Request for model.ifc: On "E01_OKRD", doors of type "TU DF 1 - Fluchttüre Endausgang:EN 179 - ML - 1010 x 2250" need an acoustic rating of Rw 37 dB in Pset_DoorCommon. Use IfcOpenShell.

First a look at what the model holds.

```python
import ifcopenshell
import ifcopenshell.util.element

model = ifcopenshell.open("model.ifc")
print(model.schema)
storey = next(s for s in model.by_type("IfcBuildingStorey") if s.Name == "E01_OKRD")
doors = [e for e in ifcopenshell.util.element.get_decomposition(storey) if e.is_a("IfcDoor")]
seen = {}
for e in doors:
    element_type = ifcopenshell.util.element.get_type(e)
    key = (element_type.Name if element_type != e and element_type else None, ifcopenshell.util.element.get_pset(e, "Pset_DoorCommon", "AcousticRating"))
    seen[key] = seen.get(key, 0) + 1
for (name, value), count in sorted(seen.items(), key=str):
    print(count, "x", name, "|", value)
```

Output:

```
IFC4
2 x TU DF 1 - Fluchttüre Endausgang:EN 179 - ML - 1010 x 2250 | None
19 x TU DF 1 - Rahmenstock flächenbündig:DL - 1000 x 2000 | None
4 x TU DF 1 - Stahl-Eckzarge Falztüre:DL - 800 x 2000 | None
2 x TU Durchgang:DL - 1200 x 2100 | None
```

```python
import ifcopenshell
import ifcopenshell.api.pset
import ifcopenshell.util.element

model = ifcopenshell.open("model.ifc")

storey = next(s for s in model.by_type("IfcBuildingStorey") if s.Name == "E01_OKRD")
doors = [e for e in ifcopenshell.util.element.get_decomposition(storey) if e.is_a("IfcDoor")]

count = 0
for e in doors:
    element_type = ifcopenshell.util.element.get_type(e)
    if element_type in (None, e) or element_type.Name != "TU DF 1 - Fluchttüre Endausgang:EN 179 - ML - 1010 x 2250":
        continue
    # add_pset returns the element's existing set when there is one.
    pset = ifcopenshell.api.pset.add_pset(model, product=e, name="Pset_DoorCommon")
    ifcopenshell.api.pset.edit_pset(model, pset=pset, properties={"AcousticRating": "Rw 37 dB"})
    count += 1

print(count, "doors updated")

model.write("model-out.ifc")
```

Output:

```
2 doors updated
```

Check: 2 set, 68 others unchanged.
